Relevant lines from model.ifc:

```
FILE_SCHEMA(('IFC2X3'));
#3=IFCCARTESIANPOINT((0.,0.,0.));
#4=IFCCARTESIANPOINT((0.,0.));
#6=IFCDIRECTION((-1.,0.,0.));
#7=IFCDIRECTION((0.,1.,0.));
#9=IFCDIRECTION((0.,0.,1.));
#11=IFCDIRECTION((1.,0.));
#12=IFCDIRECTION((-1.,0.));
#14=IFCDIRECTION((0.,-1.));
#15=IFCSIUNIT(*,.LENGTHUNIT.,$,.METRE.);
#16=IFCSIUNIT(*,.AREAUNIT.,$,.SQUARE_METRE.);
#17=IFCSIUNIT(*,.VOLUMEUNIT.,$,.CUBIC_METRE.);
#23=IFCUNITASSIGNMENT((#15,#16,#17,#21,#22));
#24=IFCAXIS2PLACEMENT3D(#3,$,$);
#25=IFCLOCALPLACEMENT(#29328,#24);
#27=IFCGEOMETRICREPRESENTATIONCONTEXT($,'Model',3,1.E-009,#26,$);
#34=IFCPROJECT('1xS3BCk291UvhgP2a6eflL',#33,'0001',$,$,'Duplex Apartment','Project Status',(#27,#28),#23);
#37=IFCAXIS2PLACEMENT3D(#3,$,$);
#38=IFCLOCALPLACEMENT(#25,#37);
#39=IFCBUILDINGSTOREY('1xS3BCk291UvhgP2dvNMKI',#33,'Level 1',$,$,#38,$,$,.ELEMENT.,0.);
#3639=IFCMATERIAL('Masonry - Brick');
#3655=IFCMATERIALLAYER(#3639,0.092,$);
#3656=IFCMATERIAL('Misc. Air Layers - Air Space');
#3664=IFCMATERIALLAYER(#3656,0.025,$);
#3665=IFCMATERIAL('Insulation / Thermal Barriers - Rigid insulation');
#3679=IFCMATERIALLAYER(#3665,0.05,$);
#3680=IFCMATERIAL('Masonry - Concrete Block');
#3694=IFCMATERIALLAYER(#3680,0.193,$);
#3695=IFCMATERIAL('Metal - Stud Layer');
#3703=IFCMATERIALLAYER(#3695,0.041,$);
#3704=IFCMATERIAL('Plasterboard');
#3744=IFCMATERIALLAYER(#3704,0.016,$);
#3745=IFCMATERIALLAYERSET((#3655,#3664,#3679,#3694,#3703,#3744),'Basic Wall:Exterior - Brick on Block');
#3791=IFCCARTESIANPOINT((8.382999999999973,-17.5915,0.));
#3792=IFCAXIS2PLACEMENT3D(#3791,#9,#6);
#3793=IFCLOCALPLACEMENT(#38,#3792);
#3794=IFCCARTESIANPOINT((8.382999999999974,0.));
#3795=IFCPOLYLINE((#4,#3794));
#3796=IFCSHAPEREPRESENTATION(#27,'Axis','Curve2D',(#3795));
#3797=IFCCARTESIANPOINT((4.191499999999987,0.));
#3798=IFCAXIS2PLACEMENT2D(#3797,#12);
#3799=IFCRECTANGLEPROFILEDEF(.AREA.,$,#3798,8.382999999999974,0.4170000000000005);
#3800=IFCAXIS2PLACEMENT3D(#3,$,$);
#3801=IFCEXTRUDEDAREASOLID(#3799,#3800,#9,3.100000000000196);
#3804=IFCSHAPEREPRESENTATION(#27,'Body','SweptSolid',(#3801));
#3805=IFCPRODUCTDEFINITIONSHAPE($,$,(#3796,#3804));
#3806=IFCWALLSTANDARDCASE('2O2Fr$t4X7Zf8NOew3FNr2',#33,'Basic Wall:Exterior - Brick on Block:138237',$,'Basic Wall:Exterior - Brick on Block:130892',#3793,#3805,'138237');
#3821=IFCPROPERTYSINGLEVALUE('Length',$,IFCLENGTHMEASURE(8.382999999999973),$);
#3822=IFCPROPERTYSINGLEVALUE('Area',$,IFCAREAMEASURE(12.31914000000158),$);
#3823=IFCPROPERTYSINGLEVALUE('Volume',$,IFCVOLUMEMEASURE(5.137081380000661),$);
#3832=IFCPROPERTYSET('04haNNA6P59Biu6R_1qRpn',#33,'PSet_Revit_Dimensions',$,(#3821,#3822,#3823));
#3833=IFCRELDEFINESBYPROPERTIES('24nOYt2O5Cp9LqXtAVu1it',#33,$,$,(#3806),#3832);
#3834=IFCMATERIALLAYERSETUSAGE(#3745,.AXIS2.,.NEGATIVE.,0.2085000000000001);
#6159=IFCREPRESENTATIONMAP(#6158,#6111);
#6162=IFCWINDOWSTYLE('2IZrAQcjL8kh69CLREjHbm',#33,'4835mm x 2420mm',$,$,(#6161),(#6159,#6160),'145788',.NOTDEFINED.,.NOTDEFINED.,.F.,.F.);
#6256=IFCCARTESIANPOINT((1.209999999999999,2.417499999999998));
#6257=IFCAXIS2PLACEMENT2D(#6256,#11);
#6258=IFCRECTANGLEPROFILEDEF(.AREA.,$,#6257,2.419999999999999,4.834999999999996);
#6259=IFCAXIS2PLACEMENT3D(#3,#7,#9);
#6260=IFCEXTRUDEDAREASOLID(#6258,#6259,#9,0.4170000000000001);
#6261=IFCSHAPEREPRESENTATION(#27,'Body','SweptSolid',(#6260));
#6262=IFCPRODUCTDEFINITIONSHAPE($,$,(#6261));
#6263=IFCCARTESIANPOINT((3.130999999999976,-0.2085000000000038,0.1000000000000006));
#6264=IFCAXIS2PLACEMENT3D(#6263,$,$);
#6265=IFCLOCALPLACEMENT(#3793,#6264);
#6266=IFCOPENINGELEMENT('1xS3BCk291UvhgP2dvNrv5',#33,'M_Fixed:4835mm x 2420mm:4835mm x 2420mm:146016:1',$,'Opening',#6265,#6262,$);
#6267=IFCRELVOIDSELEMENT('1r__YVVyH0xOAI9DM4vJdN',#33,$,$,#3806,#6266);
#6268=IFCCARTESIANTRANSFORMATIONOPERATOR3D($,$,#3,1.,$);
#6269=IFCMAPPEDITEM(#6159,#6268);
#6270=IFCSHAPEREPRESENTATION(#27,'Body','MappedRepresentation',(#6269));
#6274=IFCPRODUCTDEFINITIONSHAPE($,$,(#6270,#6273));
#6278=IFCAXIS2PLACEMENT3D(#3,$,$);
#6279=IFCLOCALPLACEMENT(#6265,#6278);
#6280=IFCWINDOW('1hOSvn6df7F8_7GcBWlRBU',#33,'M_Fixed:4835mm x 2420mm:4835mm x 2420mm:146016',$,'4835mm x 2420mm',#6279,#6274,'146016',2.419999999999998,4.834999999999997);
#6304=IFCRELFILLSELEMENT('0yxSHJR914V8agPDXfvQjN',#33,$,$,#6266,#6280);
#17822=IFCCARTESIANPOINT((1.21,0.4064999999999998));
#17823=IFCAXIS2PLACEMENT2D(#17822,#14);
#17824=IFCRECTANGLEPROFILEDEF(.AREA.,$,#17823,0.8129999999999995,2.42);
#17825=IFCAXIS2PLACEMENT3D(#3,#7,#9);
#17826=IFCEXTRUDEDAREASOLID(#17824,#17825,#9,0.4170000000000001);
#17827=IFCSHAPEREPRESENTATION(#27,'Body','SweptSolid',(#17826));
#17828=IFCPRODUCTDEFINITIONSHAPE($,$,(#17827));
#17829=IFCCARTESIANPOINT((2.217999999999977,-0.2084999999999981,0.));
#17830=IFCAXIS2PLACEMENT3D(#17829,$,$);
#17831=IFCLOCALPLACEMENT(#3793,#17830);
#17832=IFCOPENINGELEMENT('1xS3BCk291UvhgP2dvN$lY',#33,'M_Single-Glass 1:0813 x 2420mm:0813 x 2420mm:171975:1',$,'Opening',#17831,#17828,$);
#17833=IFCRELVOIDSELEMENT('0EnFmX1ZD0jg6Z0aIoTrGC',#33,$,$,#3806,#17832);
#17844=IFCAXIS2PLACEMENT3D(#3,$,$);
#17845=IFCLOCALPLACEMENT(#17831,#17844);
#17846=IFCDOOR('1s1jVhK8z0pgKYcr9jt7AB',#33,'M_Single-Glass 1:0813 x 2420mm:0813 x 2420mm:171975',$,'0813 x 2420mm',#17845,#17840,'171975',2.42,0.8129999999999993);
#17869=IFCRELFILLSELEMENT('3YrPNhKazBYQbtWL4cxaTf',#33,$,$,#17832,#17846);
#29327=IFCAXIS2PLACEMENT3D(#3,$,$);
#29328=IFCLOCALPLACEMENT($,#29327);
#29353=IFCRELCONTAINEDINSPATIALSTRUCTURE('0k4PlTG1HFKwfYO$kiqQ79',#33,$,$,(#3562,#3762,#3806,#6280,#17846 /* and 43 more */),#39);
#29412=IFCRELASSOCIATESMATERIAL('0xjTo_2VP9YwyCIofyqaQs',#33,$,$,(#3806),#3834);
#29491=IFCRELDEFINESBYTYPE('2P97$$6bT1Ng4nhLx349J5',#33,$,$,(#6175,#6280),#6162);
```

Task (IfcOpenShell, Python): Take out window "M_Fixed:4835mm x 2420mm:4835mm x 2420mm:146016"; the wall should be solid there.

```python
import ifcopenshell
import ifcopenshell.api.feature
import ifcopenshell.api.pset
import ifcopenshell.api.root
import ifcopenshell.geom
import ifcopenshell.util.element
import ifcopenshell.util.shape
import ifcopenshell.util.unit

model = ifcopenshell.open("model.ifc")
area_scale = ifcopenshell.util.unit.calculate_unit_scale(model, "AREAUNIT")
volume_scale = ifcopenshell.util.unit.calculate_unit_scale(model, "VOLUMEUNIT")
settings = ifcopenshell.geom.settings()


def volume(element):
    """Net volume in cubic metres, openings subtracted."""
    shape = ifcopenshell.geom.create_shape(settings, element)
    return ifcopenshell.util.shape.get_volume(shape.geometry)


window = model.by_guid("1hOSvn6df7F8_7GcBWlRBU")
opening = window.FillsVoids[0].RelatingOpeningElement
wall = opening.VoidsElements[0].RelatingBuildingElement
before = volume(wall)

ifcopenshell.api.root.remove_product(model, product=window)
ifcopenshell.api.feature.remove_feature(model, feature=opening)

after = volume(wall)
thickness = 0.417  # wall thickness in metres

# Update the wall's stored quantities.
pset = model.by_id(ifcopenshell.util.element.get_pset(wall, "PSet_Revit_Dimensions", should_inherit=False)["id"])
ifcopenshell.api.pset.edit_pset(model, pset=pset, properties={
    "Area": model.create_entity("IfcAreaMeasure", after / thickness / area_scale),
    "Volume": model.create_entity("IfcVolumeMeasure", after / volume_scale),
})

print(f"wall volume {before:.3f} -> {after:.3f} m3")

model.write("model_v2.ifc")
```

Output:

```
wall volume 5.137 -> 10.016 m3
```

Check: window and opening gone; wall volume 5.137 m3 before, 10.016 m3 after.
